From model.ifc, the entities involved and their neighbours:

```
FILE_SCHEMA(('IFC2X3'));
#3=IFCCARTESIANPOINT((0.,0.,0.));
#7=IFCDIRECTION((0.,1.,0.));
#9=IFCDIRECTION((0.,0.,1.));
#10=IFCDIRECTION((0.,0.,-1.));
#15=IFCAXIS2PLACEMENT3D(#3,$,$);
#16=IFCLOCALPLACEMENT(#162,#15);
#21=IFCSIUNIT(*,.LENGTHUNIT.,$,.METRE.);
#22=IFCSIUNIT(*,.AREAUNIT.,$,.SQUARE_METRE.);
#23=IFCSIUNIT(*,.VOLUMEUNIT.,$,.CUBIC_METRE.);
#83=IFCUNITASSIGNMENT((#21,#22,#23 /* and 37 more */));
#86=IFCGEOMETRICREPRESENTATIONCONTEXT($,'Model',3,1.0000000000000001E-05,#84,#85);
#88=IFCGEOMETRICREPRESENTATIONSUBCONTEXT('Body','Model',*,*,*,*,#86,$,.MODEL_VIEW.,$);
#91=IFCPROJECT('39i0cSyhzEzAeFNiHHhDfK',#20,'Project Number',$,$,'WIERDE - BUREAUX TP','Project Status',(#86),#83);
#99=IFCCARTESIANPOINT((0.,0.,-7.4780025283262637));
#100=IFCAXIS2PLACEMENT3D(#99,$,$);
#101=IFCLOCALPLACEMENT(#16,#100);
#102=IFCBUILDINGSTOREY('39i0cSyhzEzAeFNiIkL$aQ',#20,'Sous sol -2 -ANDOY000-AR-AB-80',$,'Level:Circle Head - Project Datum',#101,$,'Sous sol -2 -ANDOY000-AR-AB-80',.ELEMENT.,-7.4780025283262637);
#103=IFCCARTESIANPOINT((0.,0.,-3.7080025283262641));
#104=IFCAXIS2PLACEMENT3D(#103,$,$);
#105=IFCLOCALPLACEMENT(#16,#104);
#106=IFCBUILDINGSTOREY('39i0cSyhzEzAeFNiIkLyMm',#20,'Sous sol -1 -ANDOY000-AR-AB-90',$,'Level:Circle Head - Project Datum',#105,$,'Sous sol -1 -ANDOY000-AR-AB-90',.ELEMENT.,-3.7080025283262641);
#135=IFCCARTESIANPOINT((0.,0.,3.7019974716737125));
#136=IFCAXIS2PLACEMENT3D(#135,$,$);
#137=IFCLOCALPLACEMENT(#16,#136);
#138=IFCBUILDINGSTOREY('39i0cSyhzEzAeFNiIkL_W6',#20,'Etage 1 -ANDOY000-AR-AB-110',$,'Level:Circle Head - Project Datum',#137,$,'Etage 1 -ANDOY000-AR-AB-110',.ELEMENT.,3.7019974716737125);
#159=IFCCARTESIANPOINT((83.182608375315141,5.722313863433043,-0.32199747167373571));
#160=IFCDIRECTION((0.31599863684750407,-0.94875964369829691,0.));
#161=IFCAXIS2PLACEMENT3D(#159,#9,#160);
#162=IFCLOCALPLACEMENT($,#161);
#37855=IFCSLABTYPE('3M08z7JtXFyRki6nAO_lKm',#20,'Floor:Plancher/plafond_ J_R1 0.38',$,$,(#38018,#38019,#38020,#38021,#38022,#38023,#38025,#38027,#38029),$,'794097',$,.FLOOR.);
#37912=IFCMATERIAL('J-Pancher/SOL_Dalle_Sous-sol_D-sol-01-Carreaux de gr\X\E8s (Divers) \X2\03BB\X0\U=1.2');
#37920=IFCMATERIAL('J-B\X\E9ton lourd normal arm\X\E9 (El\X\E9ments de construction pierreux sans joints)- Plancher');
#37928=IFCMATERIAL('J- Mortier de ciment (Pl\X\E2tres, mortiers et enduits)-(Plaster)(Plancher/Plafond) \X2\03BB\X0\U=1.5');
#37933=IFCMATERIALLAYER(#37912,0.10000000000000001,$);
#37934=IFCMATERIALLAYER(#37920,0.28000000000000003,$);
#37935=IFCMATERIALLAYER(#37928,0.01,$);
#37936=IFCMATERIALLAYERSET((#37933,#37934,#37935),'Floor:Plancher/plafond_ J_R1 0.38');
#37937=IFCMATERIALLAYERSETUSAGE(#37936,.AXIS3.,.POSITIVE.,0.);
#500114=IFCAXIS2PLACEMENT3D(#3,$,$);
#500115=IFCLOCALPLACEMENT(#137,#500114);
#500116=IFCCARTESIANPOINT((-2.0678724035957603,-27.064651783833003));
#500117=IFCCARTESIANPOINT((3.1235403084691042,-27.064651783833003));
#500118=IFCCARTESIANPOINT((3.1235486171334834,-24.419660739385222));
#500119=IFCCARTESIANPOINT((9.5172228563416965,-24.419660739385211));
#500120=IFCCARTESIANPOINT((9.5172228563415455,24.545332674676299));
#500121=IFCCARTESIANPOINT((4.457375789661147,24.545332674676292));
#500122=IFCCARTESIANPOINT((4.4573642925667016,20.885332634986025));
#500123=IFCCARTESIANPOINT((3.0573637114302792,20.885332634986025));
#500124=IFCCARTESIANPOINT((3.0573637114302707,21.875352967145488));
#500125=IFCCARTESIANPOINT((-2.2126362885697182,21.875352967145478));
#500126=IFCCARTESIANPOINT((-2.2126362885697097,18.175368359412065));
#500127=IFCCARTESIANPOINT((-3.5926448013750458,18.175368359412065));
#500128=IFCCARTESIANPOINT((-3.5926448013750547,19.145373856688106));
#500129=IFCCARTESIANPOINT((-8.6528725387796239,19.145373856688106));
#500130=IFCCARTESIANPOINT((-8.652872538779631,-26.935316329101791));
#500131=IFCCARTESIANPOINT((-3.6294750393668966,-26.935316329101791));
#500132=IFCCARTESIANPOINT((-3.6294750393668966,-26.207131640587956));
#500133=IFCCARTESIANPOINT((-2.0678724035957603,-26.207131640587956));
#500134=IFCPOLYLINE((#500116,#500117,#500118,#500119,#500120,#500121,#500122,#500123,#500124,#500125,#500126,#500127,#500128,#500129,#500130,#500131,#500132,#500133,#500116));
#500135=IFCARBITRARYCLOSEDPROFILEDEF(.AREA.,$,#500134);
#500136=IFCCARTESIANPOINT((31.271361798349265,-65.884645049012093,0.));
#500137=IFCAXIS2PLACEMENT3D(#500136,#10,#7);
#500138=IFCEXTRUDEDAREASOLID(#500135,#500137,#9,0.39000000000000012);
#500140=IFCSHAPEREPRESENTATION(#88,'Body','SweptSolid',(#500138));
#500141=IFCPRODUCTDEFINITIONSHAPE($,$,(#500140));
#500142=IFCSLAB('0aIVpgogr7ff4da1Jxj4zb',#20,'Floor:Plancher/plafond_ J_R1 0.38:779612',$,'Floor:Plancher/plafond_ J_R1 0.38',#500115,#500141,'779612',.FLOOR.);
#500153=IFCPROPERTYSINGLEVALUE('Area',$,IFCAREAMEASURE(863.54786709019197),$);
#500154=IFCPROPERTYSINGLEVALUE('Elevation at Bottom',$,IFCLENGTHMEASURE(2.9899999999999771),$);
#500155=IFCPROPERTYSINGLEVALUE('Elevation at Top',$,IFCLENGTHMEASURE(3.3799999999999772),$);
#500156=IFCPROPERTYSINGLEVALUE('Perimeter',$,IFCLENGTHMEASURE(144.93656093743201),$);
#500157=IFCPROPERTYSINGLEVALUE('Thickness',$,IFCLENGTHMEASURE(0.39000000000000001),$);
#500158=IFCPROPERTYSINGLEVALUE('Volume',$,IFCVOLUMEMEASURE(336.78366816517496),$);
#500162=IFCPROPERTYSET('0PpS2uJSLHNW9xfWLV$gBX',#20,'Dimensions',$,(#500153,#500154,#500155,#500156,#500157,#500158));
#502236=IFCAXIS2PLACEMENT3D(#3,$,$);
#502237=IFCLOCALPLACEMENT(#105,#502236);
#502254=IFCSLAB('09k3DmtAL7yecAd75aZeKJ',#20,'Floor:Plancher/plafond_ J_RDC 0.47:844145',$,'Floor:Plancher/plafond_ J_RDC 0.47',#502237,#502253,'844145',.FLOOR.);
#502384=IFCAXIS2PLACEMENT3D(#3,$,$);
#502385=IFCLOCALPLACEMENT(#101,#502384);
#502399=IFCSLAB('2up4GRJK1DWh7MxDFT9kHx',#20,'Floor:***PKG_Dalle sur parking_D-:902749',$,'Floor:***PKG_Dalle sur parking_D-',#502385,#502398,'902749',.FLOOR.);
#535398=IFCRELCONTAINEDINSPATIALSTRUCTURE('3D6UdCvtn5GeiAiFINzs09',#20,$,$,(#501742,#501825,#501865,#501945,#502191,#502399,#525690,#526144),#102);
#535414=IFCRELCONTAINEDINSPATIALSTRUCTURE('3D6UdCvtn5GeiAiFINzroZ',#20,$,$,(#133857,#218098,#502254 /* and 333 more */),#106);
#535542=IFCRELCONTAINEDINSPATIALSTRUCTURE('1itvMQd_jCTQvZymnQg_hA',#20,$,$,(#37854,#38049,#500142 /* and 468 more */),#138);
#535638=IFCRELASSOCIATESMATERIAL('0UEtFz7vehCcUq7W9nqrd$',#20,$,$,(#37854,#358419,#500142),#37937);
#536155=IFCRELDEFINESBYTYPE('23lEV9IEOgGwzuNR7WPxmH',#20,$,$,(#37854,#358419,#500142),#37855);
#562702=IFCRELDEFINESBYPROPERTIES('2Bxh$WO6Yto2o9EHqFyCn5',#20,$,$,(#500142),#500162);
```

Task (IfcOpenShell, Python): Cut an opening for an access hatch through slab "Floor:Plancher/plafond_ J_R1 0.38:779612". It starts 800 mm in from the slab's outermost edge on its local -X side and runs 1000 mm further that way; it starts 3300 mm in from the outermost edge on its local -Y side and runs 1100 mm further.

```python
import numpy as np
import ifcopenshell
import ifcopenshell.api.feature
import ifcopenshell.api.geometry
import ifcopenshell.api.pset
import ifcopenshell.api.root
import ifcopenshell.geom
import ifcopenshell.util.element
import ifcopenshell.util.placement
import ifcopenshell.util.representation
import ifcopenshell.util.shape
import ifcopenshell.util.unit

model = ifcopenshell.open("model.ifc")
unit_scale = ifcopenshell.util.unit.calculate_unit_scale(model)
area_scale = ifcopenshell.util.unit.calculate_unit_scale(model, "AREAUNIT")
volume_scale = ifcopenshell.util.unit.calculate_unit_scale(model, "VOLUMEUNIT")
settings = ifcopenshell.geom.settings()


def volume(element):
    """Net volume in cubic metres, openings subtracted."""
    shape = ifcopenshell.geom.create_shape(settings, element)
    return ifcopenshell.util.shape.get_volume(shape.geometry)


slab = model.by_guid("0aIVpgogr7ff4da1Jxj4zb")
before = volume(slab)

# Extent in the slab's own axes, in metres. The edges named are its -X and -Y sides.
slab_shape = ifcopenshell.geom.create_shape(settings, slab)
vertices = ifcopenshell.util.shape.get_vertices(slab_shape.geometry)
x_min, y_min, bottom = vertices.min(axis=0)
top = vertices[:, 2].max()

opening = ifcopenshell.api.root.create_entity(model, ifc_class="IfcOpeningElement", name="Access hatch opening")
context = ifcopenshell.util.representation.get_context(model, "Model", "Body", "MODEL_VIEW")
width, depth = 1, 1.1
outline = [(0.0, 0.0), (width, 0.0), (width, depth), (0.0, depth), (0.0, 0.0)]
# Overshoot both faces by 50 mm so the cut is clean.
shape = ifcopenshell.api.geometry.add_slab_representation(
    model, context=context, depth=top - bottom + 0.1, polyline=outline
)
ifcopenshell.api.geometry.assign_representation(model, product=opening, representation=shape)

matrix = ifcopenshell.util.placement.get_local_placement(slab.ObjectPlacement)
matrix[:, 3] = matrix @ np.append(np.array([x_min + 0.8, y_min + 3.3, bottom - 0.05]) / unit_scale, 1.0)
ifcopenshell.api.geometry.edit_object_placement(model, product=opening, matrix=matrix, is_si=False)
ifcopenshell.api.feature.add_feature(model, feature=opening, element=slab)

after = volume(slab)

# Update the slab's stored quantities.
pset = model.by_id(ifcopenshell.util.element.get_pset(slab, "Dimensions", should_inherit=False)["id"])
ifcopenshell.api.pset.edit_pset(model, pset=pset, properties={
    "Area": model.create_entity("IfcAreaMeasure", after / (top - bottom) / area_scale),
    "Volume": model.create_entity("IfcVolumeMeasure", after / volume_scale),
})

print(f"slab volume {before:.3f} -> {after:.3f} m3")

model.write("model_v2.ifc")
```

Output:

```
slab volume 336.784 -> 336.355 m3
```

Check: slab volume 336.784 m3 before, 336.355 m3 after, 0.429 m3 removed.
